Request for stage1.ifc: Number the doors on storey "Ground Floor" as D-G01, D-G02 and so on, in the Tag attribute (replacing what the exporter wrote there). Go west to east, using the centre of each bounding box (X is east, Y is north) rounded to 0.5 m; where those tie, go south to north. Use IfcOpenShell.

First a look at what the model holds.

```python
import ifcopenshell
import ifcopenshell.util.element
import ifcopenshell.util.placement

model = ifcopenshell.open("stage1.ifc")
print(model.schema)
storey = next(s for s in model.by_type("IfcBuildingStorey") if s.Name == "Ground Floor")
doors = [e for e in ifcopenshell.util.element.get_decomposition(storey) if e.is_a("IfcDoor")]
for e in sorted(doors, key=lambda e: e.id()):
    origin = ifcopenshell.util.placement.get_local_placement(e.ObjectPlacement)[:3, 3]
    print(e.id(), e.Tag, e.Name, origin.round(2) + 0.0, sep=" | ")
```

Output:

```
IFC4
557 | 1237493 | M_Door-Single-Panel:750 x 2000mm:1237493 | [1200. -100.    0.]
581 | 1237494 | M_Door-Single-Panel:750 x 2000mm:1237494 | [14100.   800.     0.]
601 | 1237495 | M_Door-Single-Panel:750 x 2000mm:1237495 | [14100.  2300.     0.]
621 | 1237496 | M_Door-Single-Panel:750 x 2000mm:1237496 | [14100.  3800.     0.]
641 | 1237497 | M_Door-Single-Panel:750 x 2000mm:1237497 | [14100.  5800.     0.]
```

```python
import ifcopenshell
import ifcopenshell.geom
import ifcopenshell.util.element
import ifcopenshell.util.shape

model = ifcopenshell.open("stage1.ifc")
settings = ifcopenshell.geom.settings()
settings.set("use-world-coords", True)


def centre(element):
    shape = ifcopenshell.geom.create_shape(settings, element)
    return ifcopenshell.util.shape.get_bbox_centroid(shape.geometry)


storey = next(s for s in model.by_type("IfcBuildingStorey") if s.Name == "Ground Floor")
doors = [e for e in ifcopenshell.util.element.get_decomposition(storey) if e.is_a("IfcDoor")]

# Insertion points can sit at a corner or the storey origin, so sort by the geometry (in metres).
centres = {e: centre(e) for e in doors}
doors.sort(key=lambda e: (round(centres[e][0] / 0.5), centres[e][1]))

for i, e in enumerate(doors, start=1):
    number = f"D-G{i:02d}"
    e.Tag = number
    print(e.id(), number)

model.write("stage1_v2.ifc")
```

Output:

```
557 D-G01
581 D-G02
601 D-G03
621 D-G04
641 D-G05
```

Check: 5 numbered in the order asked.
